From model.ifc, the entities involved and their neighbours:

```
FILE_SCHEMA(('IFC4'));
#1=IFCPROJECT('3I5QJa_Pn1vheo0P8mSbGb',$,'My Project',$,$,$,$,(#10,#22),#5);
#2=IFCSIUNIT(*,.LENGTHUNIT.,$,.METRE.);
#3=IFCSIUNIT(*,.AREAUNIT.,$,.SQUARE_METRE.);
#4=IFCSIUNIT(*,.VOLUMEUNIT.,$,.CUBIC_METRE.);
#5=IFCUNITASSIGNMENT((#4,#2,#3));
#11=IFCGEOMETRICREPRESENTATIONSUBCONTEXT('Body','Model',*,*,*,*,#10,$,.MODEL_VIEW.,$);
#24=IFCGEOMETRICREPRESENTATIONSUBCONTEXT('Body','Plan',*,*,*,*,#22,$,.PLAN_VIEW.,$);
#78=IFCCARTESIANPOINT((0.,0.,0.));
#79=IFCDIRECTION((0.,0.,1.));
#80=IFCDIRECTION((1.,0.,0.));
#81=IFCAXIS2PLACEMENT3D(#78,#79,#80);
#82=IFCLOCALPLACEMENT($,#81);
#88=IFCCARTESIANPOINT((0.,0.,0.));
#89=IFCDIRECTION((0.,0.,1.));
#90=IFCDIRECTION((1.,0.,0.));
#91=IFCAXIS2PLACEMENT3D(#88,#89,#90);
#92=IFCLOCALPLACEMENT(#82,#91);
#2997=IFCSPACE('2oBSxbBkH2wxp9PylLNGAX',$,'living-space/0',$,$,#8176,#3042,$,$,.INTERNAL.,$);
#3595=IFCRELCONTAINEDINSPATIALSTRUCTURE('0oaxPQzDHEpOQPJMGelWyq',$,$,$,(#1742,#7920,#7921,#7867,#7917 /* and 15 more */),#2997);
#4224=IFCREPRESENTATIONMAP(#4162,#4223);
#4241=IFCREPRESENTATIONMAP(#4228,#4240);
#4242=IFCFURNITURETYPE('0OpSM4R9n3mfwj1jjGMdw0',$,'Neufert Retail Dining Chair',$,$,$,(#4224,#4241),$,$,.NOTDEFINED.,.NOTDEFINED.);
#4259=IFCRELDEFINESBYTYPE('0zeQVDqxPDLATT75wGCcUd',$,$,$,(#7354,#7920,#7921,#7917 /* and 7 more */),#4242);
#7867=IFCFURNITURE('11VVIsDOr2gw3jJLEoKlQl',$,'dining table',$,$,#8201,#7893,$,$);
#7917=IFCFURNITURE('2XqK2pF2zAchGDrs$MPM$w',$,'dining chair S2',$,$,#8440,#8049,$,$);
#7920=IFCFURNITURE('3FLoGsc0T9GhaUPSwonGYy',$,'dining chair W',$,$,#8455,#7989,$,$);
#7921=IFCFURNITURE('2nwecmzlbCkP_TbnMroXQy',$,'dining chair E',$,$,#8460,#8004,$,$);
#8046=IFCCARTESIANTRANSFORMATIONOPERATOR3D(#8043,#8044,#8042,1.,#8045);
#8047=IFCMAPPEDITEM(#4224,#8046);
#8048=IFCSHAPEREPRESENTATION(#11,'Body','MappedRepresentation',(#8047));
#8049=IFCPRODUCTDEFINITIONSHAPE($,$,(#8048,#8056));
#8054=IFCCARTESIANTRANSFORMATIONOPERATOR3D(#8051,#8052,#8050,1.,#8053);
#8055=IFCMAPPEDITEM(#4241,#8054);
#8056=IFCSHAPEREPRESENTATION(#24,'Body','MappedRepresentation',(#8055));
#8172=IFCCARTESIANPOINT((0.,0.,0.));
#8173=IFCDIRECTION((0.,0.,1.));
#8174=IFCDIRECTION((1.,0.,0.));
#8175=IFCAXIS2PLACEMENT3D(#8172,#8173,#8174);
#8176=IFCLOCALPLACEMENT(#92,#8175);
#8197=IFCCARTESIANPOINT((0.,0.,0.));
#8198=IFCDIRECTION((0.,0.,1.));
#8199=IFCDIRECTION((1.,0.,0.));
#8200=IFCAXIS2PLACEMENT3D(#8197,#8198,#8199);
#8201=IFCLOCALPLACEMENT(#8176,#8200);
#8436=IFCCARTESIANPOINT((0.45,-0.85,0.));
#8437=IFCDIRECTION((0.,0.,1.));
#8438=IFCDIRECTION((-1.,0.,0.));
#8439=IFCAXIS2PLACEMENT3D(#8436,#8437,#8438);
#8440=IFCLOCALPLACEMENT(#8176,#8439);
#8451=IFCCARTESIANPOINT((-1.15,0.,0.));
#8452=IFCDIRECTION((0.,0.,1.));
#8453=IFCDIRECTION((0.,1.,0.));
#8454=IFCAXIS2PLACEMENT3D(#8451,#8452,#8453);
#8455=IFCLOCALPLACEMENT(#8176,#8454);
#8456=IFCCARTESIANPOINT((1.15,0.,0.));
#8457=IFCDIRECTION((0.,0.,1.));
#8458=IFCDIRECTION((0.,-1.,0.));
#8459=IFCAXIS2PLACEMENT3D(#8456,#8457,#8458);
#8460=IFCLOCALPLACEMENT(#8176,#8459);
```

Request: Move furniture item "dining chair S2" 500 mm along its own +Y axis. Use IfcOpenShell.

```python
import ifcopenshell
import ifcopenshell.api.geometry
import ifcopenshell.util.placement
import ifcopenshell.util.unit

model = ifcopenshell.open("model.ifc")
unit_scale = ifcopenshell.util.unit.calculate_unit_scale(model)

item = model.by_id(7917)
matrix = ifcopenshell.util.placement.get_local_placement(item.ObjectPlacement)
matrix[:3, 3] += matrix[:3, 1] * 0.5 / unit_scale
ifcopenshell.api.geometry.edit_object_placement(model, product=item, matrix=matrix, is_si=False)

print(ifcopenshell.util.placement.get_local_placement(item.ObjectPlacement).round(3) + 0.0)

model.write("model_rev.ifc")
```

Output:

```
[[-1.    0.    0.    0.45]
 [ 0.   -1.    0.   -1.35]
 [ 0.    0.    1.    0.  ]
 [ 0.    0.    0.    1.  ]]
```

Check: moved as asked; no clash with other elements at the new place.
